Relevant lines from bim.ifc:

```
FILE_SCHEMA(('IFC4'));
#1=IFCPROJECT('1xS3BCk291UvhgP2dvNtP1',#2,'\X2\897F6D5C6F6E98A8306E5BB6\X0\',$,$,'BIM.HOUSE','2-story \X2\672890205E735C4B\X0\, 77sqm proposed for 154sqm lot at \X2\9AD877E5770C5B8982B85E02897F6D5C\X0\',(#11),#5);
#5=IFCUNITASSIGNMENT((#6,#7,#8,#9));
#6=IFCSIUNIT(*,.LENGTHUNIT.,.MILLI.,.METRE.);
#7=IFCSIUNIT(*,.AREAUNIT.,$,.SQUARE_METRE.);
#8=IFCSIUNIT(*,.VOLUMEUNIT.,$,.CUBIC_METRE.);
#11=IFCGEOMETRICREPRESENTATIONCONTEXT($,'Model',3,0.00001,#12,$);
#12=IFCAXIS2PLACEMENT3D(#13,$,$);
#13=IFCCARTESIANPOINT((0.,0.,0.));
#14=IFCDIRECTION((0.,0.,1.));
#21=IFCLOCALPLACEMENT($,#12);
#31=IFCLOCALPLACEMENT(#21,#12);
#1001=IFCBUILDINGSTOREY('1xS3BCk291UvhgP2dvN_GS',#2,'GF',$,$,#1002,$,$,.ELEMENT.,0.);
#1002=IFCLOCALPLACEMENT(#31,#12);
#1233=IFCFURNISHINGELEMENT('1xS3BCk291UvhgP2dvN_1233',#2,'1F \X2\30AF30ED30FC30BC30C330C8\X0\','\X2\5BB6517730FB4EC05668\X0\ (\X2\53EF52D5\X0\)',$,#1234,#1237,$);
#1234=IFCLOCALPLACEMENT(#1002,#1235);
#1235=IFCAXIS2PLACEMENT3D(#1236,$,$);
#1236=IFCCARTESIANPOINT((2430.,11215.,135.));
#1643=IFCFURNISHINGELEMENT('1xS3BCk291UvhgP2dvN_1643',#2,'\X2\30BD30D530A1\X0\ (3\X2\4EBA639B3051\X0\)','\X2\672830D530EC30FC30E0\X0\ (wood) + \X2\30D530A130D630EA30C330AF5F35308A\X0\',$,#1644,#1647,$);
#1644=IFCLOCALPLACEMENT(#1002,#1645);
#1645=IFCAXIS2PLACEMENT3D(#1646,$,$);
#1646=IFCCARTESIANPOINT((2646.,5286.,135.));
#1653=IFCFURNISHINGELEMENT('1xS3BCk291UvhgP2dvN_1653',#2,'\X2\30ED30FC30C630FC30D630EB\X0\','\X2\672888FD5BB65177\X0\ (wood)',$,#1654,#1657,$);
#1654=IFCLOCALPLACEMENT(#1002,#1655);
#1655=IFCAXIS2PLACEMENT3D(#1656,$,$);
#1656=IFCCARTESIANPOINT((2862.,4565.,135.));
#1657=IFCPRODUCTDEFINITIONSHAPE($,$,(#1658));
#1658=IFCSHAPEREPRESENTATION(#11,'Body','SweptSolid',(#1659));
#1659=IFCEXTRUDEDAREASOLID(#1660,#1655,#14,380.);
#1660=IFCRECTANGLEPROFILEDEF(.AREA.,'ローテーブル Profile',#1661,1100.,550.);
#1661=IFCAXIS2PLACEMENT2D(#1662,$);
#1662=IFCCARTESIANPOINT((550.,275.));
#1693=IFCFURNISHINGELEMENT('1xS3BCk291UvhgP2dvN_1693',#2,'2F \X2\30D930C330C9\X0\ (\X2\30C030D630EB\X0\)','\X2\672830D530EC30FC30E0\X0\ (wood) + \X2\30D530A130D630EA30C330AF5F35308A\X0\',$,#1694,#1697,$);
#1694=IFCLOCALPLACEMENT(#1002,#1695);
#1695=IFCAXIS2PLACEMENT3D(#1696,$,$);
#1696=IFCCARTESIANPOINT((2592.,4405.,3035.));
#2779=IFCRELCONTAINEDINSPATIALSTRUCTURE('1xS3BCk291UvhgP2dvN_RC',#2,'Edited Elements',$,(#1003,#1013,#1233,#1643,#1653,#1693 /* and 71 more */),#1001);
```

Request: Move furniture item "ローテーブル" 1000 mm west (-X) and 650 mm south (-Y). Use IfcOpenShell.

```python
import ifcopenshell
import ifcopenshell.api.geometry
import ifcopenshell.util.placement
import ifcopenshell.util.unit

model = ifcopenshell.open("bim.ifc")
unit_scale = ifcopenshell.util.unit.calculate_unit_scale(model)

item = model.by_guid("1xS3BCk291UvhgP2dvN_1653")
matrix = ifcopenshell.util.placement.get_local_placement(item.ObjectPlacement)
matrix[0, 3] -= 1 / unit_scale
matrix[1, 3] -= 0.65 / unit_scale
ifcopenshell.api.geometry.edit_object_placement(model, product=item, matrix=matrix, is_si=False)

print(ifcopenshell.util.placement.get_local_placement(item.ObjectPlacement).round(3) + 0.0)

model.write("bim_rev.ifc")
```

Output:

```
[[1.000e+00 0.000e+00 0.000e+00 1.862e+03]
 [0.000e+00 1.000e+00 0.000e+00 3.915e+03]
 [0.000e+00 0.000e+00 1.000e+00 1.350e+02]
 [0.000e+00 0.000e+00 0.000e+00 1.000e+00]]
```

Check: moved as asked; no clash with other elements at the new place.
